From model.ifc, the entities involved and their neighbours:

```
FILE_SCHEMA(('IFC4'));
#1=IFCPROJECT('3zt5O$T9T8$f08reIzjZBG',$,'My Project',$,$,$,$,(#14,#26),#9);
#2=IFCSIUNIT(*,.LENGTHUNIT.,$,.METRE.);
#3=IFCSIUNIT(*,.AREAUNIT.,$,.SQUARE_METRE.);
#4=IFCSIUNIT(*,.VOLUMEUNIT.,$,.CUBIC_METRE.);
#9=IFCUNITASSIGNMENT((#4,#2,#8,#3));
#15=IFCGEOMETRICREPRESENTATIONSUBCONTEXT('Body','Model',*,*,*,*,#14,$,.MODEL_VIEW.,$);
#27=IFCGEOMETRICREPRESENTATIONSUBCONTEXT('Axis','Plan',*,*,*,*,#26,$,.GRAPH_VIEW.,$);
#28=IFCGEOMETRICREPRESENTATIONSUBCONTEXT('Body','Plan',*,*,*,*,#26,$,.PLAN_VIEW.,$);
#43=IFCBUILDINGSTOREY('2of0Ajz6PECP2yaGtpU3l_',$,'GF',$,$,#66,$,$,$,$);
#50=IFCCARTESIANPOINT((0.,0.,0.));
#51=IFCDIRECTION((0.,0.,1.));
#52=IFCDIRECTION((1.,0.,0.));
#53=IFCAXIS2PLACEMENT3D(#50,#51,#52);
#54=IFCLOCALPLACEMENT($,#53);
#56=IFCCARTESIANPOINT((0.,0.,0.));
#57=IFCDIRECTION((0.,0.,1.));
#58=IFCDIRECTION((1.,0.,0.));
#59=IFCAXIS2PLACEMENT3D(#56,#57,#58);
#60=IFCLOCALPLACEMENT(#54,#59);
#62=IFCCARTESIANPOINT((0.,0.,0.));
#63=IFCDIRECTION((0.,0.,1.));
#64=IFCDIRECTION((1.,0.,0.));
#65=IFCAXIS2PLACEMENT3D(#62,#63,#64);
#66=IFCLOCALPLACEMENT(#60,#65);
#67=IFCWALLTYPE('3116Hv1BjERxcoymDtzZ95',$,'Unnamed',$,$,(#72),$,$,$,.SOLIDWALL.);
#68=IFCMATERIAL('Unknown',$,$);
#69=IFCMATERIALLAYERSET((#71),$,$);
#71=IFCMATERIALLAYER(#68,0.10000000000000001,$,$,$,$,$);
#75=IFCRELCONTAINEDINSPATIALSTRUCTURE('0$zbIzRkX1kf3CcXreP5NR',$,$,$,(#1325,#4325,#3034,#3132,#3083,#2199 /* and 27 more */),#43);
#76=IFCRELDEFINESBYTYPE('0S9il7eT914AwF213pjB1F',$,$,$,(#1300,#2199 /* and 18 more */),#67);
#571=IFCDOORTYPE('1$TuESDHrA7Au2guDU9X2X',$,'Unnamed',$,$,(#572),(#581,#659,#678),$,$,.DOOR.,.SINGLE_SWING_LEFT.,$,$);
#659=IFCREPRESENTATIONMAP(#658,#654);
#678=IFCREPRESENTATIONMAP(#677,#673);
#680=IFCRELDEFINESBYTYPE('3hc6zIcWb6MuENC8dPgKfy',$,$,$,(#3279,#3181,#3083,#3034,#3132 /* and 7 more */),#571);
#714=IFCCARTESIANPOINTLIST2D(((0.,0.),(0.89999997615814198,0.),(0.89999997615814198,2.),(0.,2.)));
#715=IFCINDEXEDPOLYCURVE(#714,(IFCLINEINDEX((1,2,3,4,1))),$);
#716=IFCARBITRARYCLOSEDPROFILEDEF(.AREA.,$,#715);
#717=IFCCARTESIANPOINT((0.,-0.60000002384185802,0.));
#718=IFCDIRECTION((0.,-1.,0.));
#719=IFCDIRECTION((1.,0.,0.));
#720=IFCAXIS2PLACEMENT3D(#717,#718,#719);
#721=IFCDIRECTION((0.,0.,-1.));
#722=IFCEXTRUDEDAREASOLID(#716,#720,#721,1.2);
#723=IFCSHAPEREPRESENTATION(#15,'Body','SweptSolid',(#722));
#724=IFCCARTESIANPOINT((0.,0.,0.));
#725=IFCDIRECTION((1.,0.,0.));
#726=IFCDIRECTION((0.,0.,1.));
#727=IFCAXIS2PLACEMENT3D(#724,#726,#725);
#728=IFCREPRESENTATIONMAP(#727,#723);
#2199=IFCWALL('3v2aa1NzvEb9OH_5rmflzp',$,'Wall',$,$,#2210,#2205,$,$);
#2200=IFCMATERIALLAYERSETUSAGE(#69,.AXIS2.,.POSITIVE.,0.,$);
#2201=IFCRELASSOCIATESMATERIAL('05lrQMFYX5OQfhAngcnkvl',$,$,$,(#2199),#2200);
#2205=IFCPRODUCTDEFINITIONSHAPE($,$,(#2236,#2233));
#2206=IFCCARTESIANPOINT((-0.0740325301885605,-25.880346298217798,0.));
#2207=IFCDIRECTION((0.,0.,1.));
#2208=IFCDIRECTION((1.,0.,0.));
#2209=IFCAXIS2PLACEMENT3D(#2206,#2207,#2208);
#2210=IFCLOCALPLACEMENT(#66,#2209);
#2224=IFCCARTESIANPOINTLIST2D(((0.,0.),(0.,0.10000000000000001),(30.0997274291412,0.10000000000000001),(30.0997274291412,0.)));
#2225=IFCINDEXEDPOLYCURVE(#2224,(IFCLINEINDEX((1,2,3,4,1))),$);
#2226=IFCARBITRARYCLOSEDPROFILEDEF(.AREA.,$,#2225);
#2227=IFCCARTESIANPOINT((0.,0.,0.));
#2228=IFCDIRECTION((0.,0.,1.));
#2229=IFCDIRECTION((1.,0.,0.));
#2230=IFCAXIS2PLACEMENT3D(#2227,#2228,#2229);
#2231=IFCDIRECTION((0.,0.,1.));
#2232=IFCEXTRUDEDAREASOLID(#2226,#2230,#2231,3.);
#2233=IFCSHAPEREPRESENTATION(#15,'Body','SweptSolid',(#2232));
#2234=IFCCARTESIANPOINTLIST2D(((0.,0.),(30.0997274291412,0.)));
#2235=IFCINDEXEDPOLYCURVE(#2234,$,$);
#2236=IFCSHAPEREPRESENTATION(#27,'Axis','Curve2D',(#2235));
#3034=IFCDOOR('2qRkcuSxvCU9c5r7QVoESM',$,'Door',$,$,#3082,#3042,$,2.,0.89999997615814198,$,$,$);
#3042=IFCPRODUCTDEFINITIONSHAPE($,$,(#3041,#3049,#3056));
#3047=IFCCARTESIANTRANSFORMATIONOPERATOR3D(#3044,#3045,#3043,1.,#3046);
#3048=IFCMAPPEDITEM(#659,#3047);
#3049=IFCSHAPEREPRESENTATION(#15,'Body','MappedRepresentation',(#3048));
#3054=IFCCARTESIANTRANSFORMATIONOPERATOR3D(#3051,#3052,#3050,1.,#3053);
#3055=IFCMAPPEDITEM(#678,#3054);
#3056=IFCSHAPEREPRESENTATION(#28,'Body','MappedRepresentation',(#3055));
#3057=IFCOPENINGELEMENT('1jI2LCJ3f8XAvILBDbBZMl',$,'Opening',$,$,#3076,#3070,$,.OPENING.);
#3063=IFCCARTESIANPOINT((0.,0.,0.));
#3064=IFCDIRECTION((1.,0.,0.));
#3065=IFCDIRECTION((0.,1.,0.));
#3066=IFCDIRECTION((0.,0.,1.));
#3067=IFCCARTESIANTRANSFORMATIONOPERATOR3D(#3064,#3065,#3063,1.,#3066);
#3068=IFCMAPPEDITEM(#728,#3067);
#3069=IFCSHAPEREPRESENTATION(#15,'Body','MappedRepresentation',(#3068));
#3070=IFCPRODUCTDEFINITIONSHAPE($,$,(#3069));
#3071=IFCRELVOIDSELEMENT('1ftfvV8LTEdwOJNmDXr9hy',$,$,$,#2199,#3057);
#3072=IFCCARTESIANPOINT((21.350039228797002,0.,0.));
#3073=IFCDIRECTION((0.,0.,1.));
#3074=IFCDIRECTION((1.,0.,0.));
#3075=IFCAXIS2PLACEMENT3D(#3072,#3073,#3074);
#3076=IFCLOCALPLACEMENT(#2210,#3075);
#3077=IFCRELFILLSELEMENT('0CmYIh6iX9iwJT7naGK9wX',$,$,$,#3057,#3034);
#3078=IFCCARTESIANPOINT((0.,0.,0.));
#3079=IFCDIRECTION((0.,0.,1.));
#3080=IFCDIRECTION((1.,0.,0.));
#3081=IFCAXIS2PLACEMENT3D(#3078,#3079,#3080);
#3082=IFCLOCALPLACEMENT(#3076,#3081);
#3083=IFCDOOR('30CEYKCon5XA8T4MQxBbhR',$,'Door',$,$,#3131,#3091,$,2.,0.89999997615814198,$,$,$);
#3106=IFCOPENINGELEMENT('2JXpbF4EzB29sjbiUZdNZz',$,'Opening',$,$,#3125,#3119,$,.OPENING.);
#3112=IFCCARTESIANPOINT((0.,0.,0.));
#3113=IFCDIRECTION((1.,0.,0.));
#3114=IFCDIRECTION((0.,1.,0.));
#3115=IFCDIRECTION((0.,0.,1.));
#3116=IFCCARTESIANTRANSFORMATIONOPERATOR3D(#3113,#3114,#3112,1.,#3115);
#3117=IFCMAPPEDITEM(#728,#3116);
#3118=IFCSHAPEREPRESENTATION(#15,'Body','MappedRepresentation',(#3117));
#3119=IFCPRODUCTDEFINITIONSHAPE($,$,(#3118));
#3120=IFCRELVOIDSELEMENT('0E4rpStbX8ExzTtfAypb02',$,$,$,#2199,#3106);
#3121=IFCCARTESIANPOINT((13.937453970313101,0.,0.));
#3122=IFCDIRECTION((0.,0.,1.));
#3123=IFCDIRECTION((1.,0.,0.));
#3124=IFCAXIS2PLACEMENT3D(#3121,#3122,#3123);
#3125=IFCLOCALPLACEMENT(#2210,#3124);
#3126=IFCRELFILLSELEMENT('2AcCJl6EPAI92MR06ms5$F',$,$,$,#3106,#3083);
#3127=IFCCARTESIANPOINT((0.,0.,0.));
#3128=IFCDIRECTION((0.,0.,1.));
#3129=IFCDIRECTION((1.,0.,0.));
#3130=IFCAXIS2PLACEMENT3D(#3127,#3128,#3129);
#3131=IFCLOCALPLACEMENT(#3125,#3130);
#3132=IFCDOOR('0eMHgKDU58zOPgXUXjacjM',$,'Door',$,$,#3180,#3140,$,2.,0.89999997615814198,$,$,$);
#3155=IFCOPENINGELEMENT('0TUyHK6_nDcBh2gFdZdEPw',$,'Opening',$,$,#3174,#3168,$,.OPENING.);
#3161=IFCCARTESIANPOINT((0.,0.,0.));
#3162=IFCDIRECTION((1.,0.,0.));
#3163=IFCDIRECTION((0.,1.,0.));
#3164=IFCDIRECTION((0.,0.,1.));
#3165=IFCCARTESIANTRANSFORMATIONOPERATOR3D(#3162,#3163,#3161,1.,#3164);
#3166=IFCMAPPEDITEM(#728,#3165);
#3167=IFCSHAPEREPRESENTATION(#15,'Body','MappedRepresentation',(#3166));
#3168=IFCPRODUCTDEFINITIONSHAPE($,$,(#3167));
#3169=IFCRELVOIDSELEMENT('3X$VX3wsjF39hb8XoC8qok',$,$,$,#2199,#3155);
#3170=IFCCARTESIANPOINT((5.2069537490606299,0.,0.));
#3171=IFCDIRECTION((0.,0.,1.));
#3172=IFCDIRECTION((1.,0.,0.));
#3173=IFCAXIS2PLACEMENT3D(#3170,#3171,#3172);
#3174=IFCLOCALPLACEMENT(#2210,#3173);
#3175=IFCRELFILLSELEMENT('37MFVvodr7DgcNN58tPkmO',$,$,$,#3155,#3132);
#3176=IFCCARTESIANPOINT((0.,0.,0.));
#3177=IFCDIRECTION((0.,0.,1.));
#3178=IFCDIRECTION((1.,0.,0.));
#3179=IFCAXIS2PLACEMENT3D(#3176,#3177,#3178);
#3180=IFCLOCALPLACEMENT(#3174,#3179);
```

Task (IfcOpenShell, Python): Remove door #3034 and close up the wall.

```python
import ifcopenshell
import ifcopenshell.api.feature
import ifcopenshell.api.root
import ifcopenshell.geom
import ifcopenshell.util.shape

model = ifcopenshell.open("model.ifc")
settings = ifcopenshell.geom.settings()


def volume(element):
    """Net volume in cubic metres, openings subtracted."""
    shape = ifcopenshell.geom.create_shape(settings, element)
    return ifcopenshell.util.shape.get_volume(shape.geometry)


door = model.by_guid("2qRkcuSxvCU9c5r7QVoESM")
opening = door.FillsVoids[0].RelatingOpeningElement
wall = opening.VoidsElements[0].RelatingBuildingElement
before = volume(wall)

ifcopenshell.api.root.remove_product(model, product=door)
ifcopenshell.api.feature.remove_feature(model, feature=opening)

after = volume(wall)

print(f"wall volume {before:.3f} -> {after:.3f} m3")

model.write("model_v2.ifc")
```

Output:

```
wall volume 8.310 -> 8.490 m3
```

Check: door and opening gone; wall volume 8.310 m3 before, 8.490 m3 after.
